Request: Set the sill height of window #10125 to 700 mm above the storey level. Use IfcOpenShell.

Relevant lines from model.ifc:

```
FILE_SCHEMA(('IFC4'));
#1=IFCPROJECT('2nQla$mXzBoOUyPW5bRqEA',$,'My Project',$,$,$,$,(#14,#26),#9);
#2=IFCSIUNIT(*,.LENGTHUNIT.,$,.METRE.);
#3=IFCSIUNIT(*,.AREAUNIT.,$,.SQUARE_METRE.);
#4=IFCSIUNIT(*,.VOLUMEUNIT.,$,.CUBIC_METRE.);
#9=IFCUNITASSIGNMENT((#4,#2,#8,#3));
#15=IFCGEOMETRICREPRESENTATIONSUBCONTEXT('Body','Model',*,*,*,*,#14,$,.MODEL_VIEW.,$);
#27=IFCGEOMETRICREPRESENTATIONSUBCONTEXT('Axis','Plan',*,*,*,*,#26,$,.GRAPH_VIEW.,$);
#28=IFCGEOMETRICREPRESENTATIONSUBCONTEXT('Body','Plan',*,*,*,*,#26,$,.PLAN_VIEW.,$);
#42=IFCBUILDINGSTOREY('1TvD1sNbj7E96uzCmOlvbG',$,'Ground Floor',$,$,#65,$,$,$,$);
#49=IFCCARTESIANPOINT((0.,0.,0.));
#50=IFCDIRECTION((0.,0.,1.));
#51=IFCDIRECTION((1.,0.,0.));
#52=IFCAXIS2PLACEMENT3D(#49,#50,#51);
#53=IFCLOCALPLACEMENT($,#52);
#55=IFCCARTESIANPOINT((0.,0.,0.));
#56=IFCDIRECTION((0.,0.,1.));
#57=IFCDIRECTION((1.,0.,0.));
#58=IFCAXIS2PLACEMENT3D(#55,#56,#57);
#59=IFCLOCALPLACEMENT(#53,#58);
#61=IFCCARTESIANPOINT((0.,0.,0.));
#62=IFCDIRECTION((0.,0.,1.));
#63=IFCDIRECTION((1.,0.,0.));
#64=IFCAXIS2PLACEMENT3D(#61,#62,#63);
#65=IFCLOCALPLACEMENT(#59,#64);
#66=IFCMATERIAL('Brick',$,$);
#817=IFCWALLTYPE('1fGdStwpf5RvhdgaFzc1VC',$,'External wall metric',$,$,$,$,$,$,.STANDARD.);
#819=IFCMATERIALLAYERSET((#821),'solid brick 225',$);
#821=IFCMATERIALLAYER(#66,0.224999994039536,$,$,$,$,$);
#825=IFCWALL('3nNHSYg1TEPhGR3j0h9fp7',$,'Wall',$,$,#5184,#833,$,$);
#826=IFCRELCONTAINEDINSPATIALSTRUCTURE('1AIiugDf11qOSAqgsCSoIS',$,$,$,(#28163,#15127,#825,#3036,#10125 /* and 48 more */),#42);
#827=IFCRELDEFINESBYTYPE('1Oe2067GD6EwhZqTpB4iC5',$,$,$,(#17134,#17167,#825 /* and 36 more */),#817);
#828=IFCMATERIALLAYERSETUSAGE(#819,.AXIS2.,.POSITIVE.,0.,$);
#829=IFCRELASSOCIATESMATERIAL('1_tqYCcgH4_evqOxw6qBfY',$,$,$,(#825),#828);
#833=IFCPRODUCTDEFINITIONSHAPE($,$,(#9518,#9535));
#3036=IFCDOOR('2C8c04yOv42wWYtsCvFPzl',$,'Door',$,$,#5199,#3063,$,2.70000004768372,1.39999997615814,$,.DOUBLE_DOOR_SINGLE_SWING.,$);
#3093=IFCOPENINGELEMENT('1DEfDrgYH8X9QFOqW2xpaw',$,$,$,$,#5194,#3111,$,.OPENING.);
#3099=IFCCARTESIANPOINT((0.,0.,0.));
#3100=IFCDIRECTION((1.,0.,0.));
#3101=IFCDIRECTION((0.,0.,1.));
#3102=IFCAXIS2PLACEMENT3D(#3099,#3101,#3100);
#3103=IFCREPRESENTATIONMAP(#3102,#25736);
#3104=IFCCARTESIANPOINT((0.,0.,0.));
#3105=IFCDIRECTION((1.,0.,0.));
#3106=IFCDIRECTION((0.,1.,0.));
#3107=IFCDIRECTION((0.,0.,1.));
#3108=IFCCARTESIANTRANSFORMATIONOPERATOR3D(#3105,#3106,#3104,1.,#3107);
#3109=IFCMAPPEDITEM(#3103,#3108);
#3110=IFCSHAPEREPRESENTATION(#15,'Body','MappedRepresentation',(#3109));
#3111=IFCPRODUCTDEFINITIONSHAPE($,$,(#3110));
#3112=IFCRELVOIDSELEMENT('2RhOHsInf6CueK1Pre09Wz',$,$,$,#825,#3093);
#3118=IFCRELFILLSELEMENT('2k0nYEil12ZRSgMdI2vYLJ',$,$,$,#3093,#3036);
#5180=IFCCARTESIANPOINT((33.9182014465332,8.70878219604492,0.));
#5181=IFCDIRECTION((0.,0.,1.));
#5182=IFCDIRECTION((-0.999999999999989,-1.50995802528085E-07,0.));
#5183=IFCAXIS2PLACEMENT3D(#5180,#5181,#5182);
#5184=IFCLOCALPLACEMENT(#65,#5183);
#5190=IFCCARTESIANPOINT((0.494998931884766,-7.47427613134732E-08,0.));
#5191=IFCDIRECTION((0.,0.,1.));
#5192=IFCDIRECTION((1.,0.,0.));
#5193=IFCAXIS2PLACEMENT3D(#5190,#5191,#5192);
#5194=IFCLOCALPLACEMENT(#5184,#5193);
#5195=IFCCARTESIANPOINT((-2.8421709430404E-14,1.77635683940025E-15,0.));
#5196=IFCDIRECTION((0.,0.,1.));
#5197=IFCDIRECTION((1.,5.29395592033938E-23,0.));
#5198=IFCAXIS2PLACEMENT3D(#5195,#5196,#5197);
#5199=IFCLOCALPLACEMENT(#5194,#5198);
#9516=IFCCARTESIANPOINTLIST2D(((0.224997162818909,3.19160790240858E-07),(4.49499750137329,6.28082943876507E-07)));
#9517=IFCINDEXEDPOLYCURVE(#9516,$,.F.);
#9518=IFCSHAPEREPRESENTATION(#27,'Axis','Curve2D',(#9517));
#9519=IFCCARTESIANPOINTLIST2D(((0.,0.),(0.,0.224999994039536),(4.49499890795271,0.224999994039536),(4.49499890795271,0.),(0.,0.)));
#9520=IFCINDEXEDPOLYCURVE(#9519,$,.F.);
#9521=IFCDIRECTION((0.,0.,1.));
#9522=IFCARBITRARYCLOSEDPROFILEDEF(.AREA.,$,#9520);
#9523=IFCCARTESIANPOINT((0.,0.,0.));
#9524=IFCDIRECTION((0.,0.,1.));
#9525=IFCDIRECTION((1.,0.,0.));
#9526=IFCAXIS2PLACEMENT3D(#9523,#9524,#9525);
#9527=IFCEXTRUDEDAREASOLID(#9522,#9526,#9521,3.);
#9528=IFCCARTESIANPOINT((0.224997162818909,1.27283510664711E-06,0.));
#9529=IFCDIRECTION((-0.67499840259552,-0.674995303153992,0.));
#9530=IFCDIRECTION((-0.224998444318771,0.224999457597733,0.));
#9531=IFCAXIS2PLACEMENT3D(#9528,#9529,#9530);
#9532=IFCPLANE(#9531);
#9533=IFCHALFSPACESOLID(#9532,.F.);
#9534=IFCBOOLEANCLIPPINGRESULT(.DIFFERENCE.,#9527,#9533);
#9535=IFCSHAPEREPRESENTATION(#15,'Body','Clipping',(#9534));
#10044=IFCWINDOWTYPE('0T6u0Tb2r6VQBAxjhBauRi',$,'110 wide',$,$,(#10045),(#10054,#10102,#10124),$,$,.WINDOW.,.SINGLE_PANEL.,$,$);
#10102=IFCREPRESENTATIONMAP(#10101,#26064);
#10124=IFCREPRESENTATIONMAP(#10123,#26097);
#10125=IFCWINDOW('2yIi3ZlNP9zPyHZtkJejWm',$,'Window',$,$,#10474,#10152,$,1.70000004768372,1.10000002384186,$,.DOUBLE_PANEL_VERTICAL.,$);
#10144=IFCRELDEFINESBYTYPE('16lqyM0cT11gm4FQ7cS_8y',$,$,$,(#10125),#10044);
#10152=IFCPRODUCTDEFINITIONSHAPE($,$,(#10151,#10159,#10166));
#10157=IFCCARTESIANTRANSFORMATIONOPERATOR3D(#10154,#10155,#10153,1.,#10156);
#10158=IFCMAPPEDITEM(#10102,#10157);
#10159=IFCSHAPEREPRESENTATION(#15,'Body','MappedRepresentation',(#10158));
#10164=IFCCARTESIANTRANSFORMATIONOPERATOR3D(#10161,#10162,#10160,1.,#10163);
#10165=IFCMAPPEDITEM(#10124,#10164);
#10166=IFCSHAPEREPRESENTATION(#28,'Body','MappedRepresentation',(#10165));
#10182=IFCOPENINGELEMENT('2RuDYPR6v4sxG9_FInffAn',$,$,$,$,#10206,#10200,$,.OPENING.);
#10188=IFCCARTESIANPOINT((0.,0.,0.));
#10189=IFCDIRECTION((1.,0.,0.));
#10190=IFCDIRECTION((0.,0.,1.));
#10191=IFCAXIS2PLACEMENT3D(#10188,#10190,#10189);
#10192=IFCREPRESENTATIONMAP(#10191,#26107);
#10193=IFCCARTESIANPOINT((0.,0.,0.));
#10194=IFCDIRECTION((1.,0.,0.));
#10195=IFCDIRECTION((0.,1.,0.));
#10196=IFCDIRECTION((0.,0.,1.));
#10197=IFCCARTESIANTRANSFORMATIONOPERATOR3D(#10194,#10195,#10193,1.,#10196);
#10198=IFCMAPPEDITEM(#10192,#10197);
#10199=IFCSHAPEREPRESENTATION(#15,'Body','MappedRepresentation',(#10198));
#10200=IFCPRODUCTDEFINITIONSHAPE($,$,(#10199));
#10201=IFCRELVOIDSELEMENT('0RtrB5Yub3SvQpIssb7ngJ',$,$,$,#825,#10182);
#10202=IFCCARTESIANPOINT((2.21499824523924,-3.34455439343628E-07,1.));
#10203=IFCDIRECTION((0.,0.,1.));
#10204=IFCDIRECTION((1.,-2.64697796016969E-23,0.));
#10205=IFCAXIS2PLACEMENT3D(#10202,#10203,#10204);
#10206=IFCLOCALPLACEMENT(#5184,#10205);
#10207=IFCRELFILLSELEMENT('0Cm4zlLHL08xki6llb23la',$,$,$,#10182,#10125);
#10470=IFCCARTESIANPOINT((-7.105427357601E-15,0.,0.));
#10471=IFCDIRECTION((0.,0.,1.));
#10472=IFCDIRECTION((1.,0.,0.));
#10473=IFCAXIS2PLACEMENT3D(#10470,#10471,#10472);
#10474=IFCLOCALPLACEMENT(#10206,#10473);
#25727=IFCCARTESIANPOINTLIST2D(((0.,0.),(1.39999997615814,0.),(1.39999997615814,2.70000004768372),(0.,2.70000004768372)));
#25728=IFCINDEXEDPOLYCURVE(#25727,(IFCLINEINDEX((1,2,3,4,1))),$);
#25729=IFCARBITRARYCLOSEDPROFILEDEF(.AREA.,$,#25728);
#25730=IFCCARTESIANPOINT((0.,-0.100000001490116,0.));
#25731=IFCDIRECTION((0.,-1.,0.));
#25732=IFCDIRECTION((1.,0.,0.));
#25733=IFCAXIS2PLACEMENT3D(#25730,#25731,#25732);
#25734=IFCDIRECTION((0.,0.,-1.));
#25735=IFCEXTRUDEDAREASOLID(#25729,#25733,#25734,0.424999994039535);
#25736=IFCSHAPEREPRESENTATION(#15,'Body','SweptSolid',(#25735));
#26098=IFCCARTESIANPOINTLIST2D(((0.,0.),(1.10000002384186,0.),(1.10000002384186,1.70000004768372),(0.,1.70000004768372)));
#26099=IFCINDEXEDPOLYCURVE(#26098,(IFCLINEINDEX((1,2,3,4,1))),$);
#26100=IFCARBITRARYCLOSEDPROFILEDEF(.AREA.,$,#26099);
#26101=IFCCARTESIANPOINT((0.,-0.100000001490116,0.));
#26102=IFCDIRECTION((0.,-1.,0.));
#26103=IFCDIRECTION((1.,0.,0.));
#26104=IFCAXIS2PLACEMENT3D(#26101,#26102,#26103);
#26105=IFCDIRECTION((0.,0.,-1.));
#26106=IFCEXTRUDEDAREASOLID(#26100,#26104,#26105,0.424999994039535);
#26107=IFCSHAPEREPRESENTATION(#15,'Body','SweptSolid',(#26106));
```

```python
import numpy as np
import ifcopenshell
import ifcopenshell.api.geometry
import ifcopenshell.geom
import ifcopenshell.util.element
import ifcopenshell.util.placement
import ifcopenshell.util.shape
import ifcopenshell.util.unit

model = ifcopenshell.open("model.ifc")
unit_scale = ifcopenshell.util.unit.calculate_unit_scale(model)

window = model.by_guid("2yIi3ZlNP9zPyHZtkJejWm")
opening = window.FillsVoids[0].RelatingOpeningElement
storey = ifcopenshell.util.element.get_container(window, ifc_class="IfcBuildingStorey")
level = ifcopenshell.util.placement.get_local_placement(storey.ObjectPlacement)[2, 3]

# The opening's origin need not be at the sill, so measure its lowest point.
shape = ifcopenshell.geom.create_shape(ifcopenshell.geom.settings(), opening)
bottom = ifcopenshell.util.shape.get_shape_bottom_elevation(shape, shape.geometry) / unit_scale
dz = level + 0.7 / unit_scale - bottom

shift = np.array([0.0, 0.0, dz])
# The window is placed relative to its opening, so it follows when the opening moves.
matrix = ifcopenshell.util.placement.get_local_placement(opening.ObjectPlacement)
matrix[:3, 3] += shift
ifcopenshell.api.geometry.edit_object_placement(
    model, product=opening, matrix=matrix, is_si=False, should_transform_children=True
)

print(f"moved by {dz * unit_scale:+.3f} m")

model.write("model_edited.ifc")
```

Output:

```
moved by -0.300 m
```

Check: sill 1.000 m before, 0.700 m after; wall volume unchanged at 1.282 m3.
